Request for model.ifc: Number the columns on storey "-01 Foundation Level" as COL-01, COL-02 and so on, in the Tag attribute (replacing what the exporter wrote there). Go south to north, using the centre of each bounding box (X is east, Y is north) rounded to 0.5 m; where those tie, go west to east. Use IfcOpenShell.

First a look at what the model holds.

```python
import ifcopenshell
import ifcopenshell.util.element
import ifcopenshell.util.placement

model = ifcopenshell.open("model.ifc")
print(model.schema)
storey = next(s for s in model.by_type("IfcBuildingStorey") if s.Name == "-01 Foundation Level")
columns = [e for e in ifcopenshell.util.element.get_decomposition(storey) if e.is_a("IfcColumn")]
for e in sorted(columns, key=lambda e: e.id()):
    origin = ifcopenshell.util.placement.get_local_placement(e.ObjectPlacement)[:3, 3]
    print(e.id(), e.Tag, e.Name, origin.round(2) + 0.0, sep=" | ")
```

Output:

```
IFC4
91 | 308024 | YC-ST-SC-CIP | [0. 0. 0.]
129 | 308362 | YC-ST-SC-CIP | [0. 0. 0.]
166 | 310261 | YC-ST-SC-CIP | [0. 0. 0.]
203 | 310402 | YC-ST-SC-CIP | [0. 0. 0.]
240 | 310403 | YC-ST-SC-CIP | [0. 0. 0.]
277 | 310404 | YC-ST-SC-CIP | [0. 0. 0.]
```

```python
import ifcopenshell
import ifcopenshell.geom
import ifcopenshell.util.element
import ifcopenshell.util.shape

model = ifcopenshell.open("model.ifc")
settings = ifcopenshell.geom.settings()
settings.set("use-world-coords", True)


def centre(element):
    shape = ifcopenshell.geom.create_shape(settings, element)
    return ifcopenshell.util.shape.get_bbox_centroid(shape.geometry)


storey = next(s for s in model.by_type("IfcBuildingStorey") if s.Name == "-01 Foundation Level")
columns = [e for e in ifcopenshell.util.element.get_decomposition(storey) if e.is_a("IfcColumn")]

# Insertion points can sit at a corner or the storey origin, so sort by the geometry (in metres).
centres = {e: centre(e) for e in columns}
columns.sort(key=lambda e: (round(centres[e][1] / 0.5), centres[e][0]))

for i, e in enumerate(columns, start=1):
    number = f"COL-{i:02d}"
    e.Tag = number
    print(e.id(), number)

model.write("model_edited.ifc")
```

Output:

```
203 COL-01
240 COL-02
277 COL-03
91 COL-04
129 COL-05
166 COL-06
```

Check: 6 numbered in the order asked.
